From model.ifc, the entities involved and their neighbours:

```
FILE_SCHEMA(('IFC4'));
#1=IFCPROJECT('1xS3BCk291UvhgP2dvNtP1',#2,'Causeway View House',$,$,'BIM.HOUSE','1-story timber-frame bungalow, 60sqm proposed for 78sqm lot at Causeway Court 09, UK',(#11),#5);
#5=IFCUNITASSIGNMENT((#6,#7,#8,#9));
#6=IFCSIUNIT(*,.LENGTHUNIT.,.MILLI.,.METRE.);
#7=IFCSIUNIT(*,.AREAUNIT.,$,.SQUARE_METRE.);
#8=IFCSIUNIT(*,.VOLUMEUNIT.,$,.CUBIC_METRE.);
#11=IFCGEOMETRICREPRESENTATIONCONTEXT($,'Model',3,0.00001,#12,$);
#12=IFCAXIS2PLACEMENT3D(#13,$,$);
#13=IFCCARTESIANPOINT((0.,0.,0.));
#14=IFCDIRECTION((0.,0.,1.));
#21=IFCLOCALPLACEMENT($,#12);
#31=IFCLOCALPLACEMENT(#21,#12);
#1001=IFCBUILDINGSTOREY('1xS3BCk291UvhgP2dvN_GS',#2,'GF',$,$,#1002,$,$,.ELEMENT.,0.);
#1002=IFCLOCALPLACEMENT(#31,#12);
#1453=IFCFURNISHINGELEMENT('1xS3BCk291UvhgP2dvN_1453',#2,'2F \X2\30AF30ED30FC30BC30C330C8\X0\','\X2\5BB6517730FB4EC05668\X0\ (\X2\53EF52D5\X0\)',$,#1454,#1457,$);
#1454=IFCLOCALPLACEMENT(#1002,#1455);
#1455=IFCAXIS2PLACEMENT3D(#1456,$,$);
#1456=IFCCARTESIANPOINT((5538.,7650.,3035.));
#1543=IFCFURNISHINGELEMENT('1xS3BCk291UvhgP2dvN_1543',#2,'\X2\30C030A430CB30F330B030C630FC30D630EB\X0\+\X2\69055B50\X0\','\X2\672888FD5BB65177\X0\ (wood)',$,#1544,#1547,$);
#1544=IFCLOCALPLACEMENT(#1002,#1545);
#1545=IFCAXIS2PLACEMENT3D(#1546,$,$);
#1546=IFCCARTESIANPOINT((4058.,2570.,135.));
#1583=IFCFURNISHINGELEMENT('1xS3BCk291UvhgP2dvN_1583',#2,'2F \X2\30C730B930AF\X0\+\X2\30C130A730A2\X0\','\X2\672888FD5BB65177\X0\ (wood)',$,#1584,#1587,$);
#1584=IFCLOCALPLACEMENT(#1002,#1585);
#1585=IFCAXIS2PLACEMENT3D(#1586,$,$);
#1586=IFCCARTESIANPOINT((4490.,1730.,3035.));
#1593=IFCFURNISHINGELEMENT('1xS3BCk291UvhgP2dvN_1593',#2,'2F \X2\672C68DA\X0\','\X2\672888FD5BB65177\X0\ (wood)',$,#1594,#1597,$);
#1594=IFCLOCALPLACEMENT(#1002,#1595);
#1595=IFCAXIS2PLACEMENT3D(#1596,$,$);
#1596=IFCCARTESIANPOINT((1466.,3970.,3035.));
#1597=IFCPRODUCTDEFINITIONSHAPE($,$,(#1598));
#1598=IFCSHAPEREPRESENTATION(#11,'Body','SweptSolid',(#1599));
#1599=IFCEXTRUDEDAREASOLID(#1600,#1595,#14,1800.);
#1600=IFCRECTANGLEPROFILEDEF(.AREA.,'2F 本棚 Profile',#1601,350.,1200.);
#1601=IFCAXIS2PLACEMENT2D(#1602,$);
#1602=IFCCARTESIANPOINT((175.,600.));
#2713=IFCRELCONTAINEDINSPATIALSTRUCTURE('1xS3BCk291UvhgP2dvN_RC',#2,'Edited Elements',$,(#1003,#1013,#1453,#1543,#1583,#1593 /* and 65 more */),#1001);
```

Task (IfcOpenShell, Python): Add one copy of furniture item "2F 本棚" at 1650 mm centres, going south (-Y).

```python
import numpy as np
import ifcopenshell
import ifcopenshell.api.geometry
import ifcopenshell.api.root
import ifcopenshell.util.element
import ifcopenshell.util.placement
import ifcopenshell.util.unit

model = ifcopenshell.open("model.ifc")
unit_scale = ifcopenshell.util.unit.calculate_unit_scale(model)


def reuse_history(source, copy):
    """copy_class also copies each property set's owner history, people and application; keep the originals."""
    for rel in copy.IsDefinedBy:
        if rel.is_a("IfcRelDefinesByProperties") and (history := rel.RelatingPropertyDefinition.OwnerHistory):
            rel.RelatingPropertyDefinition.OwnerHistory = source.OwnerHistory
            ifcopenshell.util.element.remove_deep2(model, history)


source = model.by_guid("1xS3BCk291UvhgP2dvN_1593")
base = ifcopenshell.util.placement.get_local_placement(source.ObjectPlacement)
step = np.array([0.0, -1.0, 0.0]) * 1.65 / unit_scale

for i in range(1, 2):
    copy = ifcopenshell.api.root.copy_class(model, product=source)
    copy.Representation = ifcopenshell.util.element.copy_deep(
        model, source.Representation, exclude=["IfcGeometricRepresentationContext", "IfcRepresentationMap"]
    )
    reuse_history(source, copy)
    matrix = base.copy()
    matrix[:3, 3] += i * step
    print("added at", matrix[:3, 3].round(3) + 0.0)
    ifcopenshell.api.geometry.edit_object_placement(model, product=copy, matrix=matrix, is_si=False)

model.write("model_edited.ifc")
```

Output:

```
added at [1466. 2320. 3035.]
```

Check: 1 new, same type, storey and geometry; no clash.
